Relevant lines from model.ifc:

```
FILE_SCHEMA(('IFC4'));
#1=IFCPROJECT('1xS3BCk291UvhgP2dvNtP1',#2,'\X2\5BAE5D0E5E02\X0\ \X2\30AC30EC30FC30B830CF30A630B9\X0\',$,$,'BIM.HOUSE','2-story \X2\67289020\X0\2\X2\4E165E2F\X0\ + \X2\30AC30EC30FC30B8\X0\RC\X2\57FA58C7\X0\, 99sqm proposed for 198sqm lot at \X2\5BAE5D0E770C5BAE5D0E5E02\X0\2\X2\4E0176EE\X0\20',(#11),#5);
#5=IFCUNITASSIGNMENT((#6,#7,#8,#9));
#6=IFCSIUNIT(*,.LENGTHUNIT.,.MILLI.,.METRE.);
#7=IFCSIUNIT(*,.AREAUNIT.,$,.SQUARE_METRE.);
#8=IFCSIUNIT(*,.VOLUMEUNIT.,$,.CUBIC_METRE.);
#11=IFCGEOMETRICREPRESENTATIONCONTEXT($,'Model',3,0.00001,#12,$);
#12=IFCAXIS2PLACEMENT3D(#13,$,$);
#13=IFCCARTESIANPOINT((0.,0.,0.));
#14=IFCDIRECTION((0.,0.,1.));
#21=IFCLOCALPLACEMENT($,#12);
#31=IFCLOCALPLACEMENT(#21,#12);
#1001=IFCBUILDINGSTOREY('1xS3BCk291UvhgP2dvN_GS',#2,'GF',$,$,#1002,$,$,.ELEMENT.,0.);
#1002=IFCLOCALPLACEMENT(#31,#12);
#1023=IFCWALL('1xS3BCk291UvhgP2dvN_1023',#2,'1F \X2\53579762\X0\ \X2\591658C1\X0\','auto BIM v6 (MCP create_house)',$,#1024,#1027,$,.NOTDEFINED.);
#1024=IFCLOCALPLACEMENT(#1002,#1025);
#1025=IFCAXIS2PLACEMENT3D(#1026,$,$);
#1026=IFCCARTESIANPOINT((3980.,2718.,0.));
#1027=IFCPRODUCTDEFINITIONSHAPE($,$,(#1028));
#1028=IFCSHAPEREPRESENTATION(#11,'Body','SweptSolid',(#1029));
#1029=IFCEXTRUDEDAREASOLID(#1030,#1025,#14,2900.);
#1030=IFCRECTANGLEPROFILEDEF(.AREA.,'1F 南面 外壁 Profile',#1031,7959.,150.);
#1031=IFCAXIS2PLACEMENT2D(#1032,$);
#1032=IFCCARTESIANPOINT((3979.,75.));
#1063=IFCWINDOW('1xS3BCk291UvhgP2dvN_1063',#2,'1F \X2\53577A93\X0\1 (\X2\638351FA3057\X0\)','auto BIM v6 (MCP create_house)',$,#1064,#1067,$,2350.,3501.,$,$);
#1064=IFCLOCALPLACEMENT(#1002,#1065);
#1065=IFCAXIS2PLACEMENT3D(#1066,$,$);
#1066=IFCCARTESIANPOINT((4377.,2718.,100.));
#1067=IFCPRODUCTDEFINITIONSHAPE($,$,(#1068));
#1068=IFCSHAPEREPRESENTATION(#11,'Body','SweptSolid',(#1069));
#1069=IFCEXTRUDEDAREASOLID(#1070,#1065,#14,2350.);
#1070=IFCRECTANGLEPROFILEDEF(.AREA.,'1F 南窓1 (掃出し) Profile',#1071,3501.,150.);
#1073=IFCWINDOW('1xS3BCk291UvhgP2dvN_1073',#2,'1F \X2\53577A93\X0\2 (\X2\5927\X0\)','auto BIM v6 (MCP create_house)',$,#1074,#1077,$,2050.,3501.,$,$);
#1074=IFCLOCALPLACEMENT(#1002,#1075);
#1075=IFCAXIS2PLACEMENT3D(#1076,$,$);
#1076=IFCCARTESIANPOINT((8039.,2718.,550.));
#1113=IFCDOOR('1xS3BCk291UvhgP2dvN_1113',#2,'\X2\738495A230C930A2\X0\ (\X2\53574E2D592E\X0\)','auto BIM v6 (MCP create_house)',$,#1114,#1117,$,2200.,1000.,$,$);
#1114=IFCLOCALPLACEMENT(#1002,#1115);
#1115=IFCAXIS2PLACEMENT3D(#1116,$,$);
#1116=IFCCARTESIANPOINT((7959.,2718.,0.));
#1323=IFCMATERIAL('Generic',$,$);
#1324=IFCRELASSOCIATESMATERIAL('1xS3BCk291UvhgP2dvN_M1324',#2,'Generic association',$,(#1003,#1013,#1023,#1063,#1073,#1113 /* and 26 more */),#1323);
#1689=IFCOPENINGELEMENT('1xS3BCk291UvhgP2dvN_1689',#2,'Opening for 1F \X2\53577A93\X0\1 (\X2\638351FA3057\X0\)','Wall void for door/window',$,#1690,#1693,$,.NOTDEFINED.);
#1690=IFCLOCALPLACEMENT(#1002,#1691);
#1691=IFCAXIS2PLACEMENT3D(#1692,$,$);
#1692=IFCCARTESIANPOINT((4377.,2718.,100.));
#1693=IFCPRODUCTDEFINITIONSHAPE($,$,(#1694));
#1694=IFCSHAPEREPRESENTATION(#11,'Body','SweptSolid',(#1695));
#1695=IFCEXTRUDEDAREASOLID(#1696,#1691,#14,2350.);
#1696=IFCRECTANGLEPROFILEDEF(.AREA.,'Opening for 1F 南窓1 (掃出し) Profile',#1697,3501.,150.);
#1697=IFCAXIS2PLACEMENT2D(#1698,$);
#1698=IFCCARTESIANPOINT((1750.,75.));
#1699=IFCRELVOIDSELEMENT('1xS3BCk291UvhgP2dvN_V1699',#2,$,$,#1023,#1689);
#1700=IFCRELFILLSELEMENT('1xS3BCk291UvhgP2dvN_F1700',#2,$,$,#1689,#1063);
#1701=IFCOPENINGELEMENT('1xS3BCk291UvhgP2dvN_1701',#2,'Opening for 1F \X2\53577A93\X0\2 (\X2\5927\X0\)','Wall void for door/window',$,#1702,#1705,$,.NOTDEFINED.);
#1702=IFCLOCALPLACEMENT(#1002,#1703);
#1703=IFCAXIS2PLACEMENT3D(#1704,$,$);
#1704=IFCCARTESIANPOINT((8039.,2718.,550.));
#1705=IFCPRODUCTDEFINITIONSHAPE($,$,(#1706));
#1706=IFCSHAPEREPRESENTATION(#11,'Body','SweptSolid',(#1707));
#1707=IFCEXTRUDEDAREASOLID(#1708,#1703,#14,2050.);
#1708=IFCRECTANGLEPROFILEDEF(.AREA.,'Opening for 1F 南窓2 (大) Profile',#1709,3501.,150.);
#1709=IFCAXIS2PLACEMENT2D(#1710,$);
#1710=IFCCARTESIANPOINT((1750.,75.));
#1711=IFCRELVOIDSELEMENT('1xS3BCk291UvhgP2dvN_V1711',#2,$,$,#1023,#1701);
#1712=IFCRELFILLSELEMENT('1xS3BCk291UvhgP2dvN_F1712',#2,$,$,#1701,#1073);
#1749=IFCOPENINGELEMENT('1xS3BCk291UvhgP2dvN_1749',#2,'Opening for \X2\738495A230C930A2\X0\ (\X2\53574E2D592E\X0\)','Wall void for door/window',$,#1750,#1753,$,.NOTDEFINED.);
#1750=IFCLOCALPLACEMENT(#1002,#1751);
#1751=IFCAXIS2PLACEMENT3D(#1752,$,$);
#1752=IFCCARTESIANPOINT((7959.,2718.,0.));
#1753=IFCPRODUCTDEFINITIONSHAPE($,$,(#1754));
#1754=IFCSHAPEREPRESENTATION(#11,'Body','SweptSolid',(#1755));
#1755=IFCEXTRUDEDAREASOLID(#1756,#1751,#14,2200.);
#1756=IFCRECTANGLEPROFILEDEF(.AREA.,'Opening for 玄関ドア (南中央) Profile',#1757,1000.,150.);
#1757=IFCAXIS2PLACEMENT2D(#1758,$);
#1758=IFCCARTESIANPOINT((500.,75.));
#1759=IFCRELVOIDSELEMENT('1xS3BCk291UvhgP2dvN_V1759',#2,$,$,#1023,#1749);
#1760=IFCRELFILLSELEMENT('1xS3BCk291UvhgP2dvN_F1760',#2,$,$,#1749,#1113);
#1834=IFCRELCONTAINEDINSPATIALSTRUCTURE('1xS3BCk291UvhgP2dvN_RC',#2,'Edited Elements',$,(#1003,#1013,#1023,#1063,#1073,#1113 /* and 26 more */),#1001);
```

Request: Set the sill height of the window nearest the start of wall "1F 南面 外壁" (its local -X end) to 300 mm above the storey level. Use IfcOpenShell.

```python
import numpy as np
import ifcopenshell
import ifcopenshell.api.geometry
import ifcopenshell.geom
import ifcopenshell.util.element
import ifcopenshell.util.placement
import ifcopenshell.util.shape
import ifcopenshell.util.unit

model = ifcopenshell.open("model.ifc")
unit_scale = ifcopenshell.util.unit.calculate_unit_scale(model)

window = model.by_id(1063)
opening = window.FillsVoids[0].RelatingOpeningElement
storey = ifcopenshell.util.element.get_container(window, ifc_class="IfcBuildingStorey")
level = ifcopenshell.util.placement.get_local_placement(storey.ObjectPlacement)[2, 3]

# The opening's origin need not be at the sill, so measure its lowest point.
shape = ifcopenshell.geom.create_shape(ifcopenshell.geom.settings(), opening)
bottom = ifcopenshell.util.shape.get_shape_bottom_elevation(shape, shape.geometry) / unit_scale
dz = level + 0.3 / unit_scale - bottom

shift = np.array([0.0, 0.0, dz])
# The window is not placed relative to its opening, so move both.
for product in (opening, window):
    matrix = ifcopenshell.util.placement.get_local_placement(product.ObjectPlacement)
    matrix[:3, 3] += shift
    ifcopenshell.api.geometry.edit_object_placement(model, product=product, matrix=matrix, is_si=False)

print(f"moved by {dz * unit_scale:+.3f} m")

model.write("model_rev.ifc")
```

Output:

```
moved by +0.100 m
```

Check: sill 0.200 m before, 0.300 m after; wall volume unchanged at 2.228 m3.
